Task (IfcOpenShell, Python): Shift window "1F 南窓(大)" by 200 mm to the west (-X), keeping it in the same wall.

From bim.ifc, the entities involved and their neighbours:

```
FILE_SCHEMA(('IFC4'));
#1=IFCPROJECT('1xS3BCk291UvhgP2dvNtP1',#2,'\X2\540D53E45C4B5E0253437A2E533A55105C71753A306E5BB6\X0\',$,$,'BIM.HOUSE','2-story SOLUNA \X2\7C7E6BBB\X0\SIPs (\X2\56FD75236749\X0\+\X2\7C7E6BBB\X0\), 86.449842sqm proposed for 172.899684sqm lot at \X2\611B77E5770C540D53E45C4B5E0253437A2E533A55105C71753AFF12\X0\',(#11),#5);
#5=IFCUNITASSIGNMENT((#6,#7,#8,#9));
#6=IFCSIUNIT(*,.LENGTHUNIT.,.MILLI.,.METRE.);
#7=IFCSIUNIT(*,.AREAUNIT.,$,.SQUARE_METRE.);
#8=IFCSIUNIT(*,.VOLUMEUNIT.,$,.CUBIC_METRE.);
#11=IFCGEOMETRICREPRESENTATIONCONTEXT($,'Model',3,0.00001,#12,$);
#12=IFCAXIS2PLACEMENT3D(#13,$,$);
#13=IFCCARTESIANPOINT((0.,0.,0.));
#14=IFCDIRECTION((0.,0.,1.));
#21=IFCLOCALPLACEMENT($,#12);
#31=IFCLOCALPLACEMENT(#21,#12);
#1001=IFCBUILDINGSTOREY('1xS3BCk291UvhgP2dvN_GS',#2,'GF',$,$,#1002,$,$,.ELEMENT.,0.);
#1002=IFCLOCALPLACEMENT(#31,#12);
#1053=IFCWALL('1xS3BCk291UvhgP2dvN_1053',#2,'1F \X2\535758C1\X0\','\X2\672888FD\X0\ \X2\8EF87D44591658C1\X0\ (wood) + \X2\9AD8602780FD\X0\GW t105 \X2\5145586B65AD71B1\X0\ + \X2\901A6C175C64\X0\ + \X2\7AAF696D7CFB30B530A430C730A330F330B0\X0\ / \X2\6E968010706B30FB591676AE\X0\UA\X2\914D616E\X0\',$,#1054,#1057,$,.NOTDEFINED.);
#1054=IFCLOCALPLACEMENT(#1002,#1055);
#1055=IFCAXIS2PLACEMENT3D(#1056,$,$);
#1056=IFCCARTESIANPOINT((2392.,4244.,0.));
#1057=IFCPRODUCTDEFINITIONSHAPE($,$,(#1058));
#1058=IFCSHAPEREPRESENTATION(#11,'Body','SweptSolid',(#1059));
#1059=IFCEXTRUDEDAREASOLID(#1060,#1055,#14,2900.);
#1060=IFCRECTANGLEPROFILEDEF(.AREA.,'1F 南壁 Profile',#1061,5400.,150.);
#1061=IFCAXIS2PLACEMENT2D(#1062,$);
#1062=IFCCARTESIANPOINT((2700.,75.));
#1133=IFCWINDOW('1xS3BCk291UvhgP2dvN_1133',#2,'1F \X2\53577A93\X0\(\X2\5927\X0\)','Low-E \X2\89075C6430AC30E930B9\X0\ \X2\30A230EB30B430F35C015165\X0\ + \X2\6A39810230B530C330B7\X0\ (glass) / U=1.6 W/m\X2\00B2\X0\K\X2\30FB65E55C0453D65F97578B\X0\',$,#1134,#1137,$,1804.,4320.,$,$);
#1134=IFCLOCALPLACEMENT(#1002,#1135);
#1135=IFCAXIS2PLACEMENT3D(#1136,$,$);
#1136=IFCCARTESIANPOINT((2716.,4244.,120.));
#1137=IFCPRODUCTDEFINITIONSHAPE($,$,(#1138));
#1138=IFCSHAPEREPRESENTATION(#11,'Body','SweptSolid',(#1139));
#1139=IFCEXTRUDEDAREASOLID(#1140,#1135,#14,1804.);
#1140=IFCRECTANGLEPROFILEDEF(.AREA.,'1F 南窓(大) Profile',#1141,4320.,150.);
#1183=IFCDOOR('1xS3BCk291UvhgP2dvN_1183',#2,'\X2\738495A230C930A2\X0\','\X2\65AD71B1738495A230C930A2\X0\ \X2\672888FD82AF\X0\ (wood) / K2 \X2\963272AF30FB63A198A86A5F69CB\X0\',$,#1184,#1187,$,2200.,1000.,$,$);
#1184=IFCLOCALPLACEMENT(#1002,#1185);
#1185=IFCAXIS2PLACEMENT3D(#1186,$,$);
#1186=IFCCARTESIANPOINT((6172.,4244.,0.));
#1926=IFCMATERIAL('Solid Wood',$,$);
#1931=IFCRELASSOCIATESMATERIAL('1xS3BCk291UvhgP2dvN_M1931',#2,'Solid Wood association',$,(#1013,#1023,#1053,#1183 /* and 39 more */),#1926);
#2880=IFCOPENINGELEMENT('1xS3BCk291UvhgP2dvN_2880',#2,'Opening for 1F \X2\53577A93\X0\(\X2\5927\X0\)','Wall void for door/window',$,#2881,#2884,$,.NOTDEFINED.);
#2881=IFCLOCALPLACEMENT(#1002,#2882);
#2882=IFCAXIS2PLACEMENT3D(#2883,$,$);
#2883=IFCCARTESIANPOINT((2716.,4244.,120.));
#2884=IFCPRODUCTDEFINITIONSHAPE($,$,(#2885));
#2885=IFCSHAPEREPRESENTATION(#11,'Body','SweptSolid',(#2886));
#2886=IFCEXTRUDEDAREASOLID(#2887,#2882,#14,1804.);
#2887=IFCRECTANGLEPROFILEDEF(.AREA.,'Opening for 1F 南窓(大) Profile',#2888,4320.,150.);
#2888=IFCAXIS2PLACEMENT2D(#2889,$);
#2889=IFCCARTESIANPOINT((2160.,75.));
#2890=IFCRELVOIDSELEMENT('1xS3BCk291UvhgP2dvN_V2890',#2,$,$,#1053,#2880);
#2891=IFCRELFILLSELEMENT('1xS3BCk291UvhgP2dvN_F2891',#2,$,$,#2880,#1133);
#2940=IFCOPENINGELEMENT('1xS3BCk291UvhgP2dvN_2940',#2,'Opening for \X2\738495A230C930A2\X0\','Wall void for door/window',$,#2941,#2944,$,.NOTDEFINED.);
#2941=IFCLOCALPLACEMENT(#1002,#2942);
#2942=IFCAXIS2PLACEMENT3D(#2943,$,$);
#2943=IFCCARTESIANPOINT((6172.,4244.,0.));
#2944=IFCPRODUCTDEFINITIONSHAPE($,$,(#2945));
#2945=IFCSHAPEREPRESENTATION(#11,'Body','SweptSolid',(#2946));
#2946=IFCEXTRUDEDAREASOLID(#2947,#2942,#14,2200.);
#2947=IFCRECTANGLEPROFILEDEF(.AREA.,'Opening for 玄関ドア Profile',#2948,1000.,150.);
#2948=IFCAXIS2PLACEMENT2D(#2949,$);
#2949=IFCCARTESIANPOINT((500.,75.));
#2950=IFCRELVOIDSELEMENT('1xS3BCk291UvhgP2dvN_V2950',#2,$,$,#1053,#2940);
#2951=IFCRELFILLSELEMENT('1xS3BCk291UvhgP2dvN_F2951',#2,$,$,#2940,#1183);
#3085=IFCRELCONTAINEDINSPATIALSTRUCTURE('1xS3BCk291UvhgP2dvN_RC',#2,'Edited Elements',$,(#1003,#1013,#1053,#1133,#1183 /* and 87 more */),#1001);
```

```python
import ifcopenshell
import ifcopenshell.api.geometry
import ifcopenshell.util.placement

model = ifcopenshell.open("bim.ifc")

window = model.by_id(1133)
opening = window.FillsVoids[0].RelatingOpeningElement
wall = opening.VoidsElements[0].RelatingBuildingElement

wall_matrix = ifcopenshell.util.placement.get_local_placement(wall.ObjectPlacement)
shift = wall_matrix[:3, 0] * -200.0
before = ifcopenshell.util.placement.get_local_placement(window.ObjectPlacement)[:3, 3].copy()

# The window is not placed relative to its opening, so move both.
for product in (opening, window):
    matrix = ifcopenshell.util.placement.get_local_placement(product.ObjectPlacement)
    matrix[:3, 3] += shift
    ifcopenshell.api.geometry.edit_object_placement(model, product=product, matrix=matrix, is_si=False)

after = ifcopenshell.util.placement.get_local_placement(window.ObjectPlacement)[:3, 3]
print("window moved by", (after - before).round(3) + 0.0)

model.write("bim-out.ifc")
```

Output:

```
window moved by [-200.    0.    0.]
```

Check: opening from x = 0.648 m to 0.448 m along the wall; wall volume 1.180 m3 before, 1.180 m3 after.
